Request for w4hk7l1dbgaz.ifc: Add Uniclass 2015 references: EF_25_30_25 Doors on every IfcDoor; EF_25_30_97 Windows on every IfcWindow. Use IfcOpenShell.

First a look at what the model holds.

```python
import ifcopenshell

model = ifcopenshell.open("w4hk7l1dbgaz.ifc")
print(model.schema)
print("classifications:", [c.Name for c in model.by_type("IfcClassification")])
for ifc_class in ("IfcDoor", "IfcRoof", "IfcStair", "IfcWall", "IfcWindow"):
    print(ifc_class, len(model.by_type(ifc_class)))
```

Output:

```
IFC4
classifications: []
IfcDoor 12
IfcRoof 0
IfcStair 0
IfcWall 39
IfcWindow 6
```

```python
import ifcopenshell
import ifcopenshell.api.classification

model = ifcopenshell.open("w4hk7l1dbgaz.ifc")

system = ifcopenshell.api.classification.add_classification(model, classification="Uniclass 2015")

codes = {
    "IfcDoor": ("EF_25_30_25", "Doors"),
    "IfcWindow": ("EF_25_30_97", "Windows"),
}
for ifc_class, (code, name) in codes.items():
    products = model.by_type(ifc_class)
    ifcopenshell.api.classification.add_reference(
        model, products=products, classification=system, identification=code, name=name
    )
    print(code, len(products))

model.write("w4hk7l1dbgaz-out.ifc")
```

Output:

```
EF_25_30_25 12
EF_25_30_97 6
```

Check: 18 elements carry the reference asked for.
